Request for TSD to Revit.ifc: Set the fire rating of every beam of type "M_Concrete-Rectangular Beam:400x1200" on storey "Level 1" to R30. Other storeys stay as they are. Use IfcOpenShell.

First a look at what the model holds.

```python
import ifcopenshell
import ifcopenshell.util.element

model = ifcopenshell.open("TSD to Revit.ifc")
print(model.schema)
storey = next(s for s in model.by_type("IfcBuildingStorey") if s.Name == "Level 1")
beams = [e for e in ifcopenshell.util.element.get_decomposition(storey) if e.is_a("IfcBeam")]
seen = {}
for e in beams:
    element_type = ifcopenshell.util.element.get_type(e)
    key = (element_type.Name if element_type != e and element_type else None, ifcopenshell.util.element.get_pset(e, "Pset_BeamCommon", "FireRating"))
    seen[key] = seen.get(key, 0) + 1
for (name, value), count in sorted(seen.items(), key=str):
    print(count, "x", name, "|", value)
```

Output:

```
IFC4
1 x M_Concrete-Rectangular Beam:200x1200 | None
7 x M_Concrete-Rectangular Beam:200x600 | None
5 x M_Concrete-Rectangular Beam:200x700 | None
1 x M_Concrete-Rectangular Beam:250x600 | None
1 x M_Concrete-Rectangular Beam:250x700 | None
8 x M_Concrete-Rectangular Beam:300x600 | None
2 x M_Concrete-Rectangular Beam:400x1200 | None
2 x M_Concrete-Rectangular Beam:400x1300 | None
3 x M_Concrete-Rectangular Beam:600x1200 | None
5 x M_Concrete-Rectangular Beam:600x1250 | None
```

```python
import ifcopenshell
import ifcopenshell.api.pset
import ifcopenshell.util.element

model = ifcopenshell.open("TSD to Revit.ifc")

storey = next(s for s in model.by_type("IfcBuildingStorey") if s.Name == "Level 1")
beams = [e for e in ifcopenshell.util.element.get_decomposition(storey) if e.is_a("IfcBeam")]

count = 0
for e in beams:
    element_type = ifcopenshell.util.element.get_type(e)
    if element_type in (None, e) or element_type.Name != "M_Concrete-Rectangular Beam:400x1200":
        continue
    # add_pset returns the element's existing set when there is one.
    pset = ifcopenshell.api.pset.add_pset(model, product=e, name="Pset_BeamCommon")
    ifcopenshell.api.pset.edit_pset(model, pset=pset, properties={"FireRating": "R30"})
    count += 1

print(count, "beams updated")

model.write("TSD to Revit_updated.ifc")
```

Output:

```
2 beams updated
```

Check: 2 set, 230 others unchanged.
